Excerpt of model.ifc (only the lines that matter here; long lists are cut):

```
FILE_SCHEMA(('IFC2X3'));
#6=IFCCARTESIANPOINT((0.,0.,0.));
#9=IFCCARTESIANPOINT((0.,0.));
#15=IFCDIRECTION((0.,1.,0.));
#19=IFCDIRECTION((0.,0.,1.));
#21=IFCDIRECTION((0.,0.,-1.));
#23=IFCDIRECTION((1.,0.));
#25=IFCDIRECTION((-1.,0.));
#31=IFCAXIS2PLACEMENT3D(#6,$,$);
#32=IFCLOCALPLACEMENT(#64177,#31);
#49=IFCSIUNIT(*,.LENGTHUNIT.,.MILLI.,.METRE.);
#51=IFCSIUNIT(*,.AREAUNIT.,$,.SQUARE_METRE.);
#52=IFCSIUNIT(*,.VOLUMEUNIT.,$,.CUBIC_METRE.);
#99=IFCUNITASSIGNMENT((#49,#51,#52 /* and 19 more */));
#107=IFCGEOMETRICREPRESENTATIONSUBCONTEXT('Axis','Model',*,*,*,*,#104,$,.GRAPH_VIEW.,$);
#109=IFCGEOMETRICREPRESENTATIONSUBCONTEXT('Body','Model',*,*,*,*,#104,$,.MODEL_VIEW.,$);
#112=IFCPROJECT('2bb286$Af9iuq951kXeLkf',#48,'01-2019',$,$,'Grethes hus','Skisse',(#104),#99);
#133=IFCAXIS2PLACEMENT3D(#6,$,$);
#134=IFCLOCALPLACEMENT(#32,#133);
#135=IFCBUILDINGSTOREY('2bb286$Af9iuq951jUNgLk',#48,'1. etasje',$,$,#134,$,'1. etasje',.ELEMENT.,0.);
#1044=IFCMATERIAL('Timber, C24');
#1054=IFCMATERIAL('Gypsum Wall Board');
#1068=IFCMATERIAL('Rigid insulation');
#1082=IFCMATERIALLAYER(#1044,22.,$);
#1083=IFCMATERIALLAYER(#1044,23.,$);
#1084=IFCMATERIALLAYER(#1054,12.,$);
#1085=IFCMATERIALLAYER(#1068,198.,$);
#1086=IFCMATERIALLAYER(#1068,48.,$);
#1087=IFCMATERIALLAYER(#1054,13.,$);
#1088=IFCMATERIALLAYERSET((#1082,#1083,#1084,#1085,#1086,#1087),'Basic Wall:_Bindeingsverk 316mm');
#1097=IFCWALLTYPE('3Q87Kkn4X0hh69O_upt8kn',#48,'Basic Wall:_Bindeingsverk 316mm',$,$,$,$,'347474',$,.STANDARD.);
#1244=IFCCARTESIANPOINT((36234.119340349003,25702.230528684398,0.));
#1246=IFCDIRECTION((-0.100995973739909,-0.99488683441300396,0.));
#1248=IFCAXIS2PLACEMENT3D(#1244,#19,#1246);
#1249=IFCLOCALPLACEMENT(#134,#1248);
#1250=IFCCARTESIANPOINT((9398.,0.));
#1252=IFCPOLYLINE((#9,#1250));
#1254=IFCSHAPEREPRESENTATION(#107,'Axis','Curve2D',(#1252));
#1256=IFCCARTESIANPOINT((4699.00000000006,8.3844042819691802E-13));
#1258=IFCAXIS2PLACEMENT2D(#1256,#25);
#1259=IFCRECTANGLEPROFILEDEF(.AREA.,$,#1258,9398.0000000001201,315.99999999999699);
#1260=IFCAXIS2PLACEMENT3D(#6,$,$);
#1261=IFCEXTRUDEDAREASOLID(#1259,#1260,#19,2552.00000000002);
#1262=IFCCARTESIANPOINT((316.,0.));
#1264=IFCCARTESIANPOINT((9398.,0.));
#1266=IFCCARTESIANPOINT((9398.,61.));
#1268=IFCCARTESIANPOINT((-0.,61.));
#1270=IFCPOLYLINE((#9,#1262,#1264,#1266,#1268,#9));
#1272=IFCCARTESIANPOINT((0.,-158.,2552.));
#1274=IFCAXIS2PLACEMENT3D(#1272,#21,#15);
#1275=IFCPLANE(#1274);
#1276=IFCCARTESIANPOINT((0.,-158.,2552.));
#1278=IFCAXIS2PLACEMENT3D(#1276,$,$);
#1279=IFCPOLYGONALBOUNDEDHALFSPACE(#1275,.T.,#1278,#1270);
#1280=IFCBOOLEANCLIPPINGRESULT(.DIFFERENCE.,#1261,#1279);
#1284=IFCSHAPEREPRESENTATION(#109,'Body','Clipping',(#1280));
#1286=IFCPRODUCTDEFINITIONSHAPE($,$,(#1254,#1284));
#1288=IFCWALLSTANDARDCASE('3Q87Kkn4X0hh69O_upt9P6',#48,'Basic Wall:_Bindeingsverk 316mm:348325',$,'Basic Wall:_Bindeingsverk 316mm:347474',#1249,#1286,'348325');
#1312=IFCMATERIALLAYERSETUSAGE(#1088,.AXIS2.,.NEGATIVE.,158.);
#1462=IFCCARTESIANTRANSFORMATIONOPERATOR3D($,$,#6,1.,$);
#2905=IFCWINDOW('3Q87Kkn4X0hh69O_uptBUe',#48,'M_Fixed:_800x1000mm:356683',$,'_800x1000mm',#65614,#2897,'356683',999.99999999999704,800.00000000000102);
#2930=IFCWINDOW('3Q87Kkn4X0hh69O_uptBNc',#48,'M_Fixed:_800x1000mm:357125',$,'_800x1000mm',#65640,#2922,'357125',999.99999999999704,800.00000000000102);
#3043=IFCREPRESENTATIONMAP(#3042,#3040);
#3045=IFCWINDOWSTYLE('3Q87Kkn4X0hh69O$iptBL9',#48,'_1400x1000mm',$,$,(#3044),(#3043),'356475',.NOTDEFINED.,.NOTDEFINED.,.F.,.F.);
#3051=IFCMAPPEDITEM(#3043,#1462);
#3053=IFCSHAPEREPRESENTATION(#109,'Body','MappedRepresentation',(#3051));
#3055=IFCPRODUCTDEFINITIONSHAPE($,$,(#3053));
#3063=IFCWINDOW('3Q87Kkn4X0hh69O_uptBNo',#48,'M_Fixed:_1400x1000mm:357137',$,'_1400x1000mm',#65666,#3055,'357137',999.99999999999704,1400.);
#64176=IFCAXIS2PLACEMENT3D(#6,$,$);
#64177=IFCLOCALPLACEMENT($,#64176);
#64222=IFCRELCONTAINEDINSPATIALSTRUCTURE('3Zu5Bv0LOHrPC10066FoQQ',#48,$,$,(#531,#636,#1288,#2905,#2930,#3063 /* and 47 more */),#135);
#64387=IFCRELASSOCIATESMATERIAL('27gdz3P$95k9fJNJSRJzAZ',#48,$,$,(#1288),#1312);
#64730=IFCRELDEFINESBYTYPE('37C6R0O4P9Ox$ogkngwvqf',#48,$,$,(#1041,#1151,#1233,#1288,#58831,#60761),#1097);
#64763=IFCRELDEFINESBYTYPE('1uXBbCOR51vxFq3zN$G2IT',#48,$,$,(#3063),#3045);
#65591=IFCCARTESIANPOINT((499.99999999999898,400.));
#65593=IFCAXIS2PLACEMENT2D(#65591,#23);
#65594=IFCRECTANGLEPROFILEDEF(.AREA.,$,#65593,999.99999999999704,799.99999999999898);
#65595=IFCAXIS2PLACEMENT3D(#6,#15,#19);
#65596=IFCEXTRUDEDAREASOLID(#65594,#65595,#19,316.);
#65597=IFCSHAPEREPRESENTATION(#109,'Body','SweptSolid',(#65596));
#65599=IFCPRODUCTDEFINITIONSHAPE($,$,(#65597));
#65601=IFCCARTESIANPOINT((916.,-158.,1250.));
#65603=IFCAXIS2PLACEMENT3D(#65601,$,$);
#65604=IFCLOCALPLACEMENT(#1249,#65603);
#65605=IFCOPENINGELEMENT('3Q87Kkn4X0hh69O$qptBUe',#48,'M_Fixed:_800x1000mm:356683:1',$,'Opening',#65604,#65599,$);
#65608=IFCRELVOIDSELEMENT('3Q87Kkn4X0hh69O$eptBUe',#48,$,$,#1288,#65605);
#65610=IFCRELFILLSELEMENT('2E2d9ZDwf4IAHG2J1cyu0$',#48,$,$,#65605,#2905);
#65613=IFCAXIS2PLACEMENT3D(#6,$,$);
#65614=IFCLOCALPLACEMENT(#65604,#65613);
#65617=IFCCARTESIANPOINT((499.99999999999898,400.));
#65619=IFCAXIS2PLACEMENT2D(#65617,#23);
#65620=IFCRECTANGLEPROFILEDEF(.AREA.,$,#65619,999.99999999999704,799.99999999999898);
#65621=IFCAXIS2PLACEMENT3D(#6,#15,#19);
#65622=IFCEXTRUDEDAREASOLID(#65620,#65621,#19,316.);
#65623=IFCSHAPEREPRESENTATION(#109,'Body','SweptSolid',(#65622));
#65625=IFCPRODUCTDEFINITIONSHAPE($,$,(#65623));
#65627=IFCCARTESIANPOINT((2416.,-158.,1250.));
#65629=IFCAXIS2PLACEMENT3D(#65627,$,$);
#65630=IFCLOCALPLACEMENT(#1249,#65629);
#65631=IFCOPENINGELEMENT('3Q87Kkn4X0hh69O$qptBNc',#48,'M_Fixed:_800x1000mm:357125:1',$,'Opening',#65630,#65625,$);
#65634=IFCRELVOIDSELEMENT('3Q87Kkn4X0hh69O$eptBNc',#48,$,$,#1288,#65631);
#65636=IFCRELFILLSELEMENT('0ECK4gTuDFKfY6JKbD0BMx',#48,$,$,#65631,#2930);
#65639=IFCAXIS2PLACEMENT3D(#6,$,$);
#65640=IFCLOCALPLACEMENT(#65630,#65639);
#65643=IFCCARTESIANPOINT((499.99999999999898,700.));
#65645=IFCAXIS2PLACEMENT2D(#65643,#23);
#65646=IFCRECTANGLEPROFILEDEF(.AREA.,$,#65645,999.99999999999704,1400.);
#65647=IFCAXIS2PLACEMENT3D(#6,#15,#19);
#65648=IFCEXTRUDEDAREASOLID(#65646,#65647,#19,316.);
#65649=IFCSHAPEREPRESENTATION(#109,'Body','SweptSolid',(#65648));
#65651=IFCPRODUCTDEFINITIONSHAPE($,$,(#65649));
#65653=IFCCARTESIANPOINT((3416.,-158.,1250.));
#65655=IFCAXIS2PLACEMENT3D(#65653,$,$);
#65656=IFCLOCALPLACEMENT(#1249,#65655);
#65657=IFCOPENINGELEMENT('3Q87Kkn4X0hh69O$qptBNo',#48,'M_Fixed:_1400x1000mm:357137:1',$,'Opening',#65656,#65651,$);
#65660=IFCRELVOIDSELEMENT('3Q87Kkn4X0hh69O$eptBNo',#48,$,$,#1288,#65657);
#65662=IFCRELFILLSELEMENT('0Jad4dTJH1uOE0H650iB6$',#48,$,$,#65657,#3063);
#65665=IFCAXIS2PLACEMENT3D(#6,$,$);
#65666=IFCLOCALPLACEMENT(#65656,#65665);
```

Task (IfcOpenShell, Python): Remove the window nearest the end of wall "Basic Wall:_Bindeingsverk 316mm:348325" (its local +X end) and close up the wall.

```python
import ifcopenshell
import ifcopenshell.api.feature
import ifcopenshell.api.root
import ifcopenshell.geom
import ifcopenshell.util.shape

model = ifcopenshell.open("model.ifc")
settings = ifcopenshell.geom.settings()


def volume(element):
    """Net volume in cubic metres, openings subtracted."""
    shape = ifcopenshell.geom.create_shape(settings, element)
    return ifcopenshell.util.shape.get_volume(shape.geometry)


window = model.by_id(3063)
opening = window.FillsVoids[0].RelatingOpeningElement
wall = opening.VoidsElements[0].RelatingBuildingElement
before = volume(wall)

ifcopenshell.api.root.remove_product(model, product=window)
ifcopenshell.api.feature.remove_feature(model, feature=opening)

after = volume(wall)

print(f"wall volume {before:.3f} -> {after:.3f} m3")

model.write("model_updated.ifc")
```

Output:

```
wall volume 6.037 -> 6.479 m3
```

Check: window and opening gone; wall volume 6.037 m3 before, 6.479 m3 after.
